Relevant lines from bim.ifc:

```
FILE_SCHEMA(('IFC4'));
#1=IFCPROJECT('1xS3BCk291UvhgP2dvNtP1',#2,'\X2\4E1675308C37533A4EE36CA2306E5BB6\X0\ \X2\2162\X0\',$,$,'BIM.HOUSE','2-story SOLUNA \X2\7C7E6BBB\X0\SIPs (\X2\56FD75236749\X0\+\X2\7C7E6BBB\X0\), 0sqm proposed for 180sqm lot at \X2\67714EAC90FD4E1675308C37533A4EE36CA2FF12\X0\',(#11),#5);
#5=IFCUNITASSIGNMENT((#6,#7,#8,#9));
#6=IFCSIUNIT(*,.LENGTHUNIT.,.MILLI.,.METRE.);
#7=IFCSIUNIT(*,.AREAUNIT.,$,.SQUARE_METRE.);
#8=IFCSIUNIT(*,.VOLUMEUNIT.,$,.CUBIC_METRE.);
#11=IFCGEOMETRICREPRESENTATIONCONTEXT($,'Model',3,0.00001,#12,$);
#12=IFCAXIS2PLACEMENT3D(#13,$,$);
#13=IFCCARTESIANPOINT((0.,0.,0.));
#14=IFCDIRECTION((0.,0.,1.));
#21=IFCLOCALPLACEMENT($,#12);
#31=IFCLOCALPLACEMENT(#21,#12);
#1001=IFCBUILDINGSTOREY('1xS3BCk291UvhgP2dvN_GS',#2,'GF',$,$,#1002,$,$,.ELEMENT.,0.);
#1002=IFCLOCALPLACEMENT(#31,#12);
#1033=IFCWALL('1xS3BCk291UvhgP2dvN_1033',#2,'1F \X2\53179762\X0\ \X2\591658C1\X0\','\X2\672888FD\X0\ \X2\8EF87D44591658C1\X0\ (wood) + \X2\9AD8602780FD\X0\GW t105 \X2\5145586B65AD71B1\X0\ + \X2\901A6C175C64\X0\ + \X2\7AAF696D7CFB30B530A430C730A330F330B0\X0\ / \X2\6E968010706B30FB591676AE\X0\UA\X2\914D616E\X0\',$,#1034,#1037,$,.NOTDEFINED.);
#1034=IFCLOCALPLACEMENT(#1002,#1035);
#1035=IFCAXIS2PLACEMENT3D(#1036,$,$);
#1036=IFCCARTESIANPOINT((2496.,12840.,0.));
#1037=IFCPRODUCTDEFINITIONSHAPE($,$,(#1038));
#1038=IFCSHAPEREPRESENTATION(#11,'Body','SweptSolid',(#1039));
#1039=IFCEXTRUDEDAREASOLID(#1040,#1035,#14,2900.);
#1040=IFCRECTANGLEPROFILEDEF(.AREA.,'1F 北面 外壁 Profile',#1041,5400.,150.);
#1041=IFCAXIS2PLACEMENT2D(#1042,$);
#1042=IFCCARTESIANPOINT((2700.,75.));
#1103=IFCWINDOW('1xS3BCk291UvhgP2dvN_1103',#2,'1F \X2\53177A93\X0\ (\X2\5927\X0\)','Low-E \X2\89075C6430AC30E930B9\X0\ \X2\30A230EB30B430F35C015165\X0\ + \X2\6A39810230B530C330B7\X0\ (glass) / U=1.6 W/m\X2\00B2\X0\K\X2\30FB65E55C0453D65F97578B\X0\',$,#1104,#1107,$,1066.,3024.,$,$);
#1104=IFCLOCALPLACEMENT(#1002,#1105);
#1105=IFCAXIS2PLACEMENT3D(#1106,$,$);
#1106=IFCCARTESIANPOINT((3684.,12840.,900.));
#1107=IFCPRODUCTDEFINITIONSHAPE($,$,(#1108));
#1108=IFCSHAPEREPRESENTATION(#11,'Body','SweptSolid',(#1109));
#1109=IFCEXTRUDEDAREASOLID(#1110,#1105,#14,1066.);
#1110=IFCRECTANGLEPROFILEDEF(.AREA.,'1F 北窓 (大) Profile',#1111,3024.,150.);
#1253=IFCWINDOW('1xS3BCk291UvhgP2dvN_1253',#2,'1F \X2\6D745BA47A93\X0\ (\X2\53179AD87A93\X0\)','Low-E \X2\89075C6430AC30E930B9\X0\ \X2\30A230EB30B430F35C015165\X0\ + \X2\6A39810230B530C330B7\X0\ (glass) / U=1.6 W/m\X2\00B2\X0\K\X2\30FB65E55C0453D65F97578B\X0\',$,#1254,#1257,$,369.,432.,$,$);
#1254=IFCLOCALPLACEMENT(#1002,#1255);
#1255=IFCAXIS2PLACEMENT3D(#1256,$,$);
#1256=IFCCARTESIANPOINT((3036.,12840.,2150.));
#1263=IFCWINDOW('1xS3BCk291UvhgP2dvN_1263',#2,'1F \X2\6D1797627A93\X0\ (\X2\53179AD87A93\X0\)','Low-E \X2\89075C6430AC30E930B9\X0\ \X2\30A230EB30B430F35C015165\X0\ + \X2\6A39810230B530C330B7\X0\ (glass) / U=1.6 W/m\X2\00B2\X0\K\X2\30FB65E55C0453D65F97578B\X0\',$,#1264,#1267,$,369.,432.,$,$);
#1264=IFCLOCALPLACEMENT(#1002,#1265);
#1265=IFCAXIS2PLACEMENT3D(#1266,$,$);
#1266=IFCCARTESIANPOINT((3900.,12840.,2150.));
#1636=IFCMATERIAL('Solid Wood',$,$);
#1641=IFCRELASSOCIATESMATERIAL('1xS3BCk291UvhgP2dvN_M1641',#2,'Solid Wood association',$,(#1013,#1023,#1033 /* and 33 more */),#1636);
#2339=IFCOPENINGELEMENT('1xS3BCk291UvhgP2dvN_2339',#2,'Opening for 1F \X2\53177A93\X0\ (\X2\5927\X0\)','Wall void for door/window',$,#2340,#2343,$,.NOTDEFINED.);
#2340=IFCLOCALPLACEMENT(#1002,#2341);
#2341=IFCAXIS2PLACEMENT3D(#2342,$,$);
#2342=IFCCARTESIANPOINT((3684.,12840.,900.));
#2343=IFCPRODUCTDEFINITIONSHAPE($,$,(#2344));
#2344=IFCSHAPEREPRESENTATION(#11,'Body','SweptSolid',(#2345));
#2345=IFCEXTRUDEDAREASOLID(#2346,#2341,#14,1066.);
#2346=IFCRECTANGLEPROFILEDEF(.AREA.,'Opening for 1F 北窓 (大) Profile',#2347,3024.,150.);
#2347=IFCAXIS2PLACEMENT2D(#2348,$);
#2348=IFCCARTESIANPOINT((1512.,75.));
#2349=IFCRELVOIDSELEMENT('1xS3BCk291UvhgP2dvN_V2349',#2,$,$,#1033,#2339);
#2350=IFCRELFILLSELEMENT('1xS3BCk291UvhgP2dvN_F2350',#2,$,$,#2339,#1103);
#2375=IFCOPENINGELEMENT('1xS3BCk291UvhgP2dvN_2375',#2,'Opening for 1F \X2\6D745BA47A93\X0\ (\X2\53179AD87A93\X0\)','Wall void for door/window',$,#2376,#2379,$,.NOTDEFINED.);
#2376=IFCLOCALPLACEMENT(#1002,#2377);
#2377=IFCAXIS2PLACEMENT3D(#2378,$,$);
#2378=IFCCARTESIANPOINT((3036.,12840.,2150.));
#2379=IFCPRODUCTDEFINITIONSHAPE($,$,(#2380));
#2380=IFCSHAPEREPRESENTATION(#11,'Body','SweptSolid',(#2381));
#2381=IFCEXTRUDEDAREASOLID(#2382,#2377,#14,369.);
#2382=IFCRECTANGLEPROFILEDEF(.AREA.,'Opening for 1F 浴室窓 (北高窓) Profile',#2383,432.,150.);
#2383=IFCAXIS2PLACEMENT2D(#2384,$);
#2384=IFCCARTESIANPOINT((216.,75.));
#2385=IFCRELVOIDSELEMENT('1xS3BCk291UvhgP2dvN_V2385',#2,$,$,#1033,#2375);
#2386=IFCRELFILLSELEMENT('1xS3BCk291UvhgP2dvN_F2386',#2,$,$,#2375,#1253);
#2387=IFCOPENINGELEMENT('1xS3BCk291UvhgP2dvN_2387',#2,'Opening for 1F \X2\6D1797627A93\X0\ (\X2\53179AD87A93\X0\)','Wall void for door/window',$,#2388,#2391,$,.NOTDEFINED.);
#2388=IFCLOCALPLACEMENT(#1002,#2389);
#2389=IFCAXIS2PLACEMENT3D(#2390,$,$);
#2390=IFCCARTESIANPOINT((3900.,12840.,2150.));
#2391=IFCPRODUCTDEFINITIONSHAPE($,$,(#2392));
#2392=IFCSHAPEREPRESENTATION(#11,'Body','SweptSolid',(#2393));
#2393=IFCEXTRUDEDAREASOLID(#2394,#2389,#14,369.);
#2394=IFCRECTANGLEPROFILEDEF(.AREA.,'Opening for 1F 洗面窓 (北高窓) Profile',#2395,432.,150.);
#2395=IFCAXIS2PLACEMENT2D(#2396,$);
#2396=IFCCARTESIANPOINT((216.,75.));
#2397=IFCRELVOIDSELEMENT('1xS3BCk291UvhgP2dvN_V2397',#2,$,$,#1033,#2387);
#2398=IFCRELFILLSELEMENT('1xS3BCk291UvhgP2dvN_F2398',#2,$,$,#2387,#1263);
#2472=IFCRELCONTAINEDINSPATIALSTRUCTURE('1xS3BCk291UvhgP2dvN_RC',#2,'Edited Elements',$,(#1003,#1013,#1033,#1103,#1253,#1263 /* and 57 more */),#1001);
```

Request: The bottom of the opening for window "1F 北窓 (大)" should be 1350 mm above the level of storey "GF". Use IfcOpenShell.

```python
import numpy as np
import ifcopenshell
import ifcopenshell.api.geometry
import ifcopenshell.geom
import ifcopenshell.util.element
import ifcopenshell.util.placement
import ifcopenshell.util.shape
import ifcopenshell.util.unit

model = ifcopenshell.open("bim.ifc")
unit_scale = ifcopenshell.util.unit.calculate_unit_scale(model)

window = model.by_guid("1xS3BCk291UvhgP2dvN_1103")
opening = window.FillsVoids[0].RelatingOpeningElement
storey = ifcopenshell.util.element.get_container(window, ifc_class="IfcBuildingStorey")
level = ifcopenshell.util.placement.get_local_placement(storey.ObjectPlacement)[2, 3]

# The opening's origin need not be at the sill, so measure its lowest point.
shape = ifcopenshell.geom.create_shape(ifcopenshell.geom.settings(), opening)
bottom = ifcopenshell.util.shape.get_shape_bottom_elevation(shape, shape.geometry) / unit_scale
dz = level + 1350.0 - bottom

shift = np.array([0.0, 0.0, dz])
# The window is not placed relative to its opening, so move both.
for product in (opening, window):
    matrix = ifcopenshell.util.placement.get_local_placement(product.ObjectPlacement)
    matrix[:3, 3] += shift
    ifcopenshell.api.geometry.edit_object_placement(model, product=product, matrix=matrix, is_si=False)

print(f"moved by {dz * unit_scale:+.3f} m")

model.write("bim_edited.ifc")
```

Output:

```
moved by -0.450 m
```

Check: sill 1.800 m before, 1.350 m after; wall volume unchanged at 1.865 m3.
